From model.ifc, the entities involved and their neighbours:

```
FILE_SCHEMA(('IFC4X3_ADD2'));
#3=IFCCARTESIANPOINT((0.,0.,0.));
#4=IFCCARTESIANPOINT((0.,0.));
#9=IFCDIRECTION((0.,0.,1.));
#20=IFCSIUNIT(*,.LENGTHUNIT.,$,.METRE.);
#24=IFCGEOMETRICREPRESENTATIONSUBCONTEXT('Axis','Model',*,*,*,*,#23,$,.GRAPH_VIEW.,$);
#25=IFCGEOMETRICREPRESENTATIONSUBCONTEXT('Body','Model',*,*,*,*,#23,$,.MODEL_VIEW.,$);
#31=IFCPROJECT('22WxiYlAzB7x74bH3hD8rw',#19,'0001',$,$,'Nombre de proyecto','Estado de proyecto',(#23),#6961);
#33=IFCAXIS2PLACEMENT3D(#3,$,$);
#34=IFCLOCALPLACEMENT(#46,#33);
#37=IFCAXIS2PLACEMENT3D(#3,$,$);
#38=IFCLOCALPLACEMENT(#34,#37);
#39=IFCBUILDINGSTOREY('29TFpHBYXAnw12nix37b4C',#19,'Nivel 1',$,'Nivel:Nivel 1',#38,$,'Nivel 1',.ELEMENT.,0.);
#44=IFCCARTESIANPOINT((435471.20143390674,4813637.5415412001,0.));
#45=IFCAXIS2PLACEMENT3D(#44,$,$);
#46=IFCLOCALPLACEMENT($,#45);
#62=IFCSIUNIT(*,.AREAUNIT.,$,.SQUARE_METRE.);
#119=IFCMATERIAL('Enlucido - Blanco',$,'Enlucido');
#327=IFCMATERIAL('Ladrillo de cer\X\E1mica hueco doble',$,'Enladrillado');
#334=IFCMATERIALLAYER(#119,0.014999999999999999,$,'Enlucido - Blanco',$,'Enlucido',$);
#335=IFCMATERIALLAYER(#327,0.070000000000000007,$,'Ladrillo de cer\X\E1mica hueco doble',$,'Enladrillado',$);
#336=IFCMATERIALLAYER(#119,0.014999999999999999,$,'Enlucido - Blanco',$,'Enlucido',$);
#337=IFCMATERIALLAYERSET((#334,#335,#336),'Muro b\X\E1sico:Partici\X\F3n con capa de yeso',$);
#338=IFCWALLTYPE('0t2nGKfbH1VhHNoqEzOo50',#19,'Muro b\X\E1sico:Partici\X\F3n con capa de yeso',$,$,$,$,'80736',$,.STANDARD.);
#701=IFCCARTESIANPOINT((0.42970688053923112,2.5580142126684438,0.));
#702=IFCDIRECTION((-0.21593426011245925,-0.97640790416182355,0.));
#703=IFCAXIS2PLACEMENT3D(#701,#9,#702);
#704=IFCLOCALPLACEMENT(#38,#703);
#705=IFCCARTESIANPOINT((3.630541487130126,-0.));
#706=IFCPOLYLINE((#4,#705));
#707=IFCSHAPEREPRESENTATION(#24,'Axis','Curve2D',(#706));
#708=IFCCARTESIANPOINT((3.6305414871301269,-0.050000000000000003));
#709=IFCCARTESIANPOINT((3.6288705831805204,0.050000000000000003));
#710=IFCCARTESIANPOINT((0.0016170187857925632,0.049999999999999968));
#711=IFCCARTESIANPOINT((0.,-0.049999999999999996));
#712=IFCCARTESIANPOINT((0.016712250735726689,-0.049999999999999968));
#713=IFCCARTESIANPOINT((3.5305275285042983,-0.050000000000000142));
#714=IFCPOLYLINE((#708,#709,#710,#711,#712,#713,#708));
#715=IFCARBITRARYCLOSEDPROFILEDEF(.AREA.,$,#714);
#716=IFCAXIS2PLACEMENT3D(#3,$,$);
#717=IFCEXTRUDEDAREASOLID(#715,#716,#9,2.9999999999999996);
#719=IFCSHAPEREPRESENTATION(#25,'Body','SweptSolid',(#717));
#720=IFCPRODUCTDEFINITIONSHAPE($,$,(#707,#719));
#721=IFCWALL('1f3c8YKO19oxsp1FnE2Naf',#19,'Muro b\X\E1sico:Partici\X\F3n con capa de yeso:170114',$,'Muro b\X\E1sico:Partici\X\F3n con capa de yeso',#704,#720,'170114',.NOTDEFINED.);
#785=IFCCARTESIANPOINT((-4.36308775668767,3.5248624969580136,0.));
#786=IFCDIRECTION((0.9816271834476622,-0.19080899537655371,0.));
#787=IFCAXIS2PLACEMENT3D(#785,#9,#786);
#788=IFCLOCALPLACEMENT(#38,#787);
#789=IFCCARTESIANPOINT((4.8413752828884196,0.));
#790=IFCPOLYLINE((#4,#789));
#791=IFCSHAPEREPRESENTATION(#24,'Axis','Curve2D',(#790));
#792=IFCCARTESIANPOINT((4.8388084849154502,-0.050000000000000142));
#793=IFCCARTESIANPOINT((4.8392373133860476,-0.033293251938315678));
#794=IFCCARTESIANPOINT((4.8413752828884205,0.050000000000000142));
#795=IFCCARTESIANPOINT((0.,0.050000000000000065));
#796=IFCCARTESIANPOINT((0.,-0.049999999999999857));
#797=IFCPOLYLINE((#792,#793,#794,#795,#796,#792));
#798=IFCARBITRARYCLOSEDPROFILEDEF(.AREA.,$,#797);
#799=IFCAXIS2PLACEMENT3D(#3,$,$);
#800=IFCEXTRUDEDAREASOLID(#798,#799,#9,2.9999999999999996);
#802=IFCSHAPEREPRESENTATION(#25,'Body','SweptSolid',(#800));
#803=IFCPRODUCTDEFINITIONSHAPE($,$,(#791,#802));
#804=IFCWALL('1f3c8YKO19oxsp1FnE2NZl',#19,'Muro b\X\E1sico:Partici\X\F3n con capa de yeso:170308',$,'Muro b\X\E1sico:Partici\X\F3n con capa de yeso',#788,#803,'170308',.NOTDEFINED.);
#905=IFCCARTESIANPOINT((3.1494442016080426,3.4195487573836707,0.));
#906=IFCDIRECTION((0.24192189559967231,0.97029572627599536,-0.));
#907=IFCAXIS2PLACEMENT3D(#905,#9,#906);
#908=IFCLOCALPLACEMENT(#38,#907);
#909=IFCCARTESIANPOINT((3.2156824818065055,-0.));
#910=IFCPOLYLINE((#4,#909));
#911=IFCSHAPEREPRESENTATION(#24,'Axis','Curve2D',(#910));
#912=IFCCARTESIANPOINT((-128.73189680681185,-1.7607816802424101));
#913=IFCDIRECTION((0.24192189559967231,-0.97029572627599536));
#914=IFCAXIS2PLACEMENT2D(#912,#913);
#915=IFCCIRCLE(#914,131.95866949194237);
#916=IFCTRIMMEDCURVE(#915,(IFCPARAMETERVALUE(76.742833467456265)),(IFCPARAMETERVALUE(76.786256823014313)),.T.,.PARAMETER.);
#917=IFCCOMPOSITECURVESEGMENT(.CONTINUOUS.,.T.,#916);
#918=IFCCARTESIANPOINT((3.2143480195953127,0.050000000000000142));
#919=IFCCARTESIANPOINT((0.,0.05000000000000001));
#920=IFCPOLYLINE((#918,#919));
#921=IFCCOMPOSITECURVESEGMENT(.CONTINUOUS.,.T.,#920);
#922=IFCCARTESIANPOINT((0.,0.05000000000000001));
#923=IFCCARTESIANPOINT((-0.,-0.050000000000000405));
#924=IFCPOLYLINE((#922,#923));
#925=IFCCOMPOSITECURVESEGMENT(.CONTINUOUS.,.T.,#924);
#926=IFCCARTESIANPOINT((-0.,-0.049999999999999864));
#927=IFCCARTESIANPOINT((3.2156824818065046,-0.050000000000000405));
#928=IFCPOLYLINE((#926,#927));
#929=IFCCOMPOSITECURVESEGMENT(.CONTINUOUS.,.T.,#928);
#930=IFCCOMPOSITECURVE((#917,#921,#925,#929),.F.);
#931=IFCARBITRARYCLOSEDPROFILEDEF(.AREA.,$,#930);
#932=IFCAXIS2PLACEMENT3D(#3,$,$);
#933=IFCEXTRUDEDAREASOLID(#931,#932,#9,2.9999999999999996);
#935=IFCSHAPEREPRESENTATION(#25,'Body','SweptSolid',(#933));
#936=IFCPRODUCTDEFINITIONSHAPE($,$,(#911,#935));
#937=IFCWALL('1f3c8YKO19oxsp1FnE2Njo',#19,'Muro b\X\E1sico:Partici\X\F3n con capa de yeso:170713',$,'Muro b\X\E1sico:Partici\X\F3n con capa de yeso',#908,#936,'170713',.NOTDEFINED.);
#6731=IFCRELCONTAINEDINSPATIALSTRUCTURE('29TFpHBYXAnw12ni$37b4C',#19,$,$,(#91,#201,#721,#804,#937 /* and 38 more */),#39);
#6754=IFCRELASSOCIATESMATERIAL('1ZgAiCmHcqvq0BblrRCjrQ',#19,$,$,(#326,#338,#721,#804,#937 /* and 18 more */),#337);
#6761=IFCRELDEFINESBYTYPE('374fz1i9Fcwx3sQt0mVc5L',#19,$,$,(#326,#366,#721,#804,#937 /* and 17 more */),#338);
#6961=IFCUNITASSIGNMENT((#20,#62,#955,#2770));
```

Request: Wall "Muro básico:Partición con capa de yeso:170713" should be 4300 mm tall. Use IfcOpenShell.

```python
import ifcopenshell
import ifcopenshell.geom
import ifcopenshell.util.representation
import ifcopenshell.util.shape
import ifcopenshell.util.unit

model = ifcopenshell.open("model.ifc")
unit_scale = ifcopenshell.util.unit.calculate_unit_scale(model)
settings = ifcopenshell.geom.settings()


def volume(element):
    """Net volume in cubic metres, openings subtracted."""
    shape = ifcopenshell.geom.create_shape(settings, element)
    return ifcopenshell.util.shape.get_volume(shape.geometry)


wall = model.by_id(937)
before = volume(wall)

body = ifcopenshell.util.representation.get_representation(wall, "Model", "Body")
solid = body.Items[0]
old_height = solid.Depth
solid.Depth = 4.3 / unit_scale
after = volume(wall)

print(f"height {old_height:g} -> {solid.Depth:g}, volume {before:.3f} -> {after:.3f} m3")

model.write("model_edited.ifc")
```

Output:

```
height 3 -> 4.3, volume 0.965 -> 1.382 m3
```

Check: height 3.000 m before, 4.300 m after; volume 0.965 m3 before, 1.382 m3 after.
